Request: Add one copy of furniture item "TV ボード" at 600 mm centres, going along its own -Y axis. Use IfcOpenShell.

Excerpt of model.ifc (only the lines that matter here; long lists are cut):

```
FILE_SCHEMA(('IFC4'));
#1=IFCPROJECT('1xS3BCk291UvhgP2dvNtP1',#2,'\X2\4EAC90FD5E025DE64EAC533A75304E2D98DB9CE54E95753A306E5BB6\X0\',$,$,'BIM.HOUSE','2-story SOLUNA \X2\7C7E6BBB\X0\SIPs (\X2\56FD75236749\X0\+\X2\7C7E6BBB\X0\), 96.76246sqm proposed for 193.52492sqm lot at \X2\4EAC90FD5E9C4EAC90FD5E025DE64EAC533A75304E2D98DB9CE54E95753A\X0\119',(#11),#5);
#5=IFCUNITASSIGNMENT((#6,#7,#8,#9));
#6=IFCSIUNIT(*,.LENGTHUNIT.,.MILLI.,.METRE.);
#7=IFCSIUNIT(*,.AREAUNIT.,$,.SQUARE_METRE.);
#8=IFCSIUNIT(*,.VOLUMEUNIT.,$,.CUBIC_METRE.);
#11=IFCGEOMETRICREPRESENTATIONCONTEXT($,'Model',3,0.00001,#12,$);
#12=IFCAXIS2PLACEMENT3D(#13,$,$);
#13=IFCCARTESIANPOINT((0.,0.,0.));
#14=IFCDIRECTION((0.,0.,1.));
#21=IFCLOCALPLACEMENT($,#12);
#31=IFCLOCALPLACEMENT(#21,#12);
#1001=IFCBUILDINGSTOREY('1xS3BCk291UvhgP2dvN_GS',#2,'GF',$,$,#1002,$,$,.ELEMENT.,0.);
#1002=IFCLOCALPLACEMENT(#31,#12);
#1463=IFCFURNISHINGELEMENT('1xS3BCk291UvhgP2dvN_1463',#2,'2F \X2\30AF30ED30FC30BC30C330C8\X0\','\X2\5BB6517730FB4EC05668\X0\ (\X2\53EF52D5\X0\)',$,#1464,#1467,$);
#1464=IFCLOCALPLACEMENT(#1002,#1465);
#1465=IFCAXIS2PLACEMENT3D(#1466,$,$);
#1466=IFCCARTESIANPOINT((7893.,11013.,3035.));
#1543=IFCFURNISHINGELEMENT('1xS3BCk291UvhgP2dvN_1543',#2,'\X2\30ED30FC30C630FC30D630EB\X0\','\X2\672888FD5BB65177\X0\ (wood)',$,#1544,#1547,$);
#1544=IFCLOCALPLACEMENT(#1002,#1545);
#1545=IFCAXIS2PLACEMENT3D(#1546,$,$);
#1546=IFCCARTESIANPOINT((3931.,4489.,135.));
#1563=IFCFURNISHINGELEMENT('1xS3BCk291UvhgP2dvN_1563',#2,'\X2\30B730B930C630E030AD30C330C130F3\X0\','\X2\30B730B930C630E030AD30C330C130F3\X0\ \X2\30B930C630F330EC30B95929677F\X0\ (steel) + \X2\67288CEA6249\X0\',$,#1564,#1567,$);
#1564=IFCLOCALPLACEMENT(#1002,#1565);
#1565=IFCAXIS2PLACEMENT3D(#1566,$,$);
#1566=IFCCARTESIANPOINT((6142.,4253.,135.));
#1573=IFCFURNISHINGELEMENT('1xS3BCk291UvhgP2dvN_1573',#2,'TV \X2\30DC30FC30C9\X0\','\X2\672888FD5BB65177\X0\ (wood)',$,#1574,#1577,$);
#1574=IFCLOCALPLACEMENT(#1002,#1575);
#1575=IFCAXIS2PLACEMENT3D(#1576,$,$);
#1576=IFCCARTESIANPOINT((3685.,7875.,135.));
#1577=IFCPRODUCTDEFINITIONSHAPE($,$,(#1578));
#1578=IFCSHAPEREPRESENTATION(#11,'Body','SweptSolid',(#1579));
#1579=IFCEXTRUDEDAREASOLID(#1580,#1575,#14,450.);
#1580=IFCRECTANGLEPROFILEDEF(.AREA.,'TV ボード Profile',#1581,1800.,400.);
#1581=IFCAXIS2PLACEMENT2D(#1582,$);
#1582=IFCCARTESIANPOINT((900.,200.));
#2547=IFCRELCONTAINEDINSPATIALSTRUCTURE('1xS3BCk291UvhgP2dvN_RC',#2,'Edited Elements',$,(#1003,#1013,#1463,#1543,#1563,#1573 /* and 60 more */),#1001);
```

```python
import ifcopenshell
import ifcopenshell.api.geometry
import ifcopenshell.api.root
import ifcopenshell.util.element
import ifcopenshell.util.placement
import ifcopenshell.util.unit

model = ifcopenshell.open("model.ifc")
unit_scale = ifcopenshell.util.unit.calculate_unit_scale(model)


def reuse_history(source, copy):
    """copy_class also copies each property set's owner history, people and application; keep the originals."""
    for rel in copy.IsDefinedBy:
        if rel.is_a("IfcRelDefinesByProperties") and (history := rel.RelatingPropertyDefinition.OwnerHistory):
            rel.RelatingPropertyDefinition.OwnerHistory = source.OwnerHistory
            ifcopenshell.util.element.remove_deep2(model, history)


source = model.by_id(1573)
base = ifcopenshell.util.placement.get_local_placement(source.ObjectPlacement)
step = -base[:3, 1] * 0.6 / unit_scale

for i in range(1, 2):
    copy = ifcopenshell.api.root.copy_class(model, product=source)
    copy.Representation = ifcopenshell.util.element.copy_deep(
        model, source.Representation, exclude=["IfcGeometricRepresentationContext", "IfcRepresentationMap"]
    )
    reuse_history(source, copy)
    matrix = base.copy()
    matrix[:3, 3] += i * step
    print("added at", matrix[:3, 3].round(3) + 0.0)
    ifcopenshell.api.geometry.edit_object_placement(model, product=copy, matrix=matrix, is_si=False)

model.write("model-out.ifc")
```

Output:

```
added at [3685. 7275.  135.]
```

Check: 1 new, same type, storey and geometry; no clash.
